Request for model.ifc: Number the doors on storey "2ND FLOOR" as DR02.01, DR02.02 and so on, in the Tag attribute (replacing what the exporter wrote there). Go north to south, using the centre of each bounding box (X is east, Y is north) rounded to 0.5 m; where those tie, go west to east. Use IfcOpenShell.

First a look at what the model holds.

```python
import ifcopenshell
import ifcopenshell.util.element
import ifcopenshell.util.placement

model = ifcopenshell.open("model.ifc")
print(model.schema)
storey = next(s for s in model.by_type("IfcBuildingStorey") if s.Name == "2ND FLOOR")
doors = [e for e in ifcopenshell.util.element.get_decomposition(storey) if e.is_a("IfcDoor")]
for e in sorted(doors, key=lambda e: e.id()):
    origin = ifcopenshell.util.placement.get_local_placement(e.ObjectPlacement)[:3, 3]
    print(e.id(), e.Tag, e.Name, origin.round(2) + 0.0, sep=" | ")
```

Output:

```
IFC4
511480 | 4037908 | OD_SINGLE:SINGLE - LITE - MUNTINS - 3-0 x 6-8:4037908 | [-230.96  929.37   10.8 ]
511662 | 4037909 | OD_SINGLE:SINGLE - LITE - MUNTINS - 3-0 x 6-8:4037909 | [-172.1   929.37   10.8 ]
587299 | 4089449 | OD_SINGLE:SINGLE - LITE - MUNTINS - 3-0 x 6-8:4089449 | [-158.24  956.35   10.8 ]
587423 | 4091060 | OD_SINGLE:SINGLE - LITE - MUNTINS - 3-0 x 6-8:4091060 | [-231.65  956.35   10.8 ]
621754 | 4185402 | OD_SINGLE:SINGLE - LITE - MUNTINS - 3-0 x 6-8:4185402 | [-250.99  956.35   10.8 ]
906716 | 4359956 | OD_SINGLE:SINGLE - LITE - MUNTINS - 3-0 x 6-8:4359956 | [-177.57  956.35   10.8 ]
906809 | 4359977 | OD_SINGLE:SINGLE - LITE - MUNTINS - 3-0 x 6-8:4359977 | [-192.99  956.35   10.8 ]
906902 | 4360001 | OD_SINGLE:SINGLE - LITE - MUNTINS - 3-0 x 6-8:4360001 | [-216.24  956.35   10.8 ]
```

```python
import ifcopenshell
import ifcopenshell.geom
import ifcopenshell.util.element
import ifcopenshell.util.shape

model = ifcopenshell.open("model.ifc")
settings = ifcopenshell.geom.settings()
settings.set("use-world-coords", True)


def centre(element):
    shape = ifcopenshell.geom.create_shape(settings, element)
    return ifcopenshell.util.shape.get_bbox_centroid(shape.geometry)


storey = next(s for s in model.by_type("IfcBuildingStorey") if s.Name == "2ND FLOOR")
doors = [e for e in ifcopenshell.util.element.get_decomposition(storey) if e.is_a("IfcDoor")]

# Insertion points can sit at a corner or the storey origin, so sort by the geometry (in metres).
centres = {e: centre(e) for e in doors}
doors.sort(key=lambda e: (-round(centres[e][1] / 0.5), centres[e][0]))

for i, e in enumerate(doors, start=1):
    number = f"DR02.{i:02d}"
    e.Tag = number
    print(e.id(), number)

model.write("model-out.ifc")
```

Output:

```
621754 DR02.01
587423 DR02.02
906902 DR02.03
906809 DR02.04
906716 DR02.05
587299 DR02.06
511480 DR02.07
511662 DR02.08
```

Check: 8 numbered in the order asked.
